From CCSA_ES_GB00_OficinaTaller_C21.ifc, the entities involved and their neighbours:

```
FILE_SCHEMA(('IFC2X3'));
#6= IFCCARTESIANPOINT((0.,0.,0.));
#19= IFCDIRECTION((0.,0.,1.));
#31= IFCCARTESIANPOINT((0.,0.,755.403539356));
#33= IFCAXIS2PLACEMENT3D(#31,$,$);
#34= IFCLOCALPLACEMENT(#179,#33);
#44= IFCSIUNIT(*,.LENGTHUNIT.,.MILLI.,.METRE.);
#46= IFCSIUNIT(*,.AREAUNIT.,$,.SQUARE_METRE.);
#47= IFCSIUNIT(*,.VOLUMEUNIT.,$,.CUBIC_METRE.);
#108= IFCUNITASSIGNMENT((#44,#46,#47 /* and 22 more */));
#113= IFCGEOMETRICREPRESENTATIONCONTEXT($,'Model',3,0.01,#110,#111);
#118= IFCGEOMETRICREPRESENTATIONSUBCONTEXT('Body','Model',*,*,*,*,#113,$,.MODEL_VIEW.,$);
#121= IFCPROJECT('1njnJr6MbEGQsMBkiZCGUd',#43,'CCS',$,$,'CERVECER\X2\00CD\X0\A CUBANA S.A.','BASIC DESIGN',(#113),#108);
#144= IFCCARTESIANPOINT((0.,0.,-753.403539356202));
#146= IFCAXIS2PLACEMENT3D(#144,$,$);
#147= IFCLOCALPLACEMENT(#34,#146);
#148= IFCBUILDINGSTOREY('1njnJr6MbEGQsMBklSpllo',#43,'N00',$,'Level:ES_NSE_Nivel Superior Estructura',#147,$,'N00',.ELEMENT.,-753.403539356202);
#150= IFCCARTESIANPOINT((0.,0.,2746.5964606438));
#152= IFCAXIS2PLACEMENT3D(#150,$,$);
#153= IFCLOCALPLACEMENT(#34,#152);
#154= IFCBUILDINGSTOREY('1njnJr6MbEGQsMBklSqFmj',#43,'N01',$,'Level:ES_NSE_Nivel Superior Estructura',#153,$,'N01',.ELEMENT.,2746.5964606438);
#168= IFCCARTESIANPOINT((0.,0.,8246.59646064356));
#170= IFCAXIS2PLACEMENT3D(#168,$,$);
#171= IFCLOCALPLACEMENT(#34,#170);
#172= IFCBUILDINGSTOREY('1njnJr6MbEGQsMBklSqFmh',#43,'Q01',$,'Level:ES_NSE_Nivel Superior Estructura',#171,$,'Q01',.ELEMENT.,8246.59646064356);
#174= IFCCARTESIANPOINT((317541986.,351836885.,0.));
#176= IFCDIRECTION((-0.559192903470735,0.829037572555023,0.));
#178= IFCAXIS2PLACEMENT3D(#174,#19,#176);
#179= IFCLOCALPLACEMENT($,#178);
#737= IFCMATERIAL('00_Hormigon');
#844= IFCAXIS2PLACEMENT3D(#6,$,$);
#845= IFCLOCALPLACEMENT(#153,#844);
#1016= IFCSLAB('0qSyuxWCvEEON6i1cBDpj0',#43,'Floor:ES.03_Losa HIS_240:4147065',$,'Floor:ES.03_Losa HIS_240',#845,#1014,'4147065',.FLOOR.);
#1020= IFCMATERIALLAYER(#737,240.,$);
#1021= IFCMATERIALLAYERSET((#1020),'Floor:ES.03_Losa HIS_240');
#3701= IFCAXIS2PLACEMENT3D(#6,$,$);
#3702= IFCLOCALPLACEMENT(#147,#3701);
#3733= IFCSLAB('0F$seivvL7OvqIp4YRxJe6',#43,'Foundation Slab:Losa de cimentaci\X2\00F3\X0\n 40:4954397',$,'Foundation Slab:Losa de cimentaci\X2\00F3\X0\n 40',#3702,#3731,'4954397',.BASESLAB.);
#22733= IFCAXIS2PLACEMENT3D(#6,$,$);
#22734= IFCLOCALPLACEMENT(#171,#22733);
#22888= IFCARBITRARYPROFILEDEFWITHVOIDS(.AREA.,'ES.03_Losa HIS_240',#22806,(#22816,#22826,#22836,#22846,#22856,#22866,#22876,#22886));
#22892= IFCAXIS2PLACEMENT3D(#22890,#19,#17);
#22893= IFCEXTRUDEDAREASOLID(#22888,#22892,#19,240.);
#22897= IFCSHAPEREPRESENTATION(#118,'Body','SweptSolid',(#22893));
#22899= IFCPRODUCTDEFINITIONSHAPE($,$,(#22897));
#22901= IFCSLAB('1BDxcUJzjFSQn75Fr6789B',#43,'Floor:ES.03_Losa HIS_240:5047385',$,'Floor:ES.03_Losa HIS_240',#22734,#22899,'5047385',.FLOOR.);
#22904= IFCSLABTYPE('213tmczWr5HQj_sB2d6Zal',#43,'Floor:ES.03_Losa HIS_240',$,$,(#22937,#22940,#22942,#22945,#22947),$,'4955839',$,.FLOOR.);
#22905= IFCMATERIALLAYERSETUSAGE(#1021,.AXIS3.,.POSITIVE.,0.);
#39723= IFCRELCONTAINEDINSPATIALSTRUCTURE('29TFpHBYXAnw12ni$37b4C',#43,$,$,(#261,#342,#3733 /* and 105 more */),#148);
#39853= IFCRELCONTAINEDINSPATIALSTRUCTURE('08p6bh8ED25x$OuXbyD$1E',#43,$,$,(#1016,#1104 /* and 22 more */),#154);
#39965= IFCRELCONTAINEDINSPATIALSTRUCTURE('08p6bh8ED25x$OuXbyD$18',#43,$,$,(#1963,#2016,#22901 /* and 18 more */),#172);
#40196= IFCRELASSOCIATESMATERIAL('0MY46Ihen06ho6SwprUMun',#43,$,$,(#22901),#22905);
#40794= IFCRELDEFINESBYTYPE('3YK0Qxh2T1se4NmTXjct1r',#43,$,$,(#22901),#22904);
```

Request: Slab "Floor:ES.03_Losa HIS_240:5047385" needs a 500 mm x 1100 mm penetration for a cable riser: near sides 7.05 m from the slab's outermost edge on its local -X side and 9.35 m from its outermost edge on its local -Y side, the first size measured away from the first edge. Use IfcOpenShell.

```python
import numpy as np
import ifcopenshell
import ifcopenshell.api.feature
import ifcopenshell.api.geometry
import ifcopenshell.api.root
import ifcopenshell.geom
import ifcopenshell.util.placement
import ifcopenshell.util.representation
import ifcopenshell.util.shape
import ifcopenshell.util.unit

model = ifcopenshell.open("CCSA_ES_GB00_OficinaTaller_C21.ifc")
unit_scale = ifcopenshell.util.unit.calculate_unit_scale(model)
settings = ifcopenshell.geom.settings()


def volume(element):
    """Net volume in cubic metres, openings subtracted."""
    shape = ifcopenshell.geom.create_shape(settings, element)
    return ifcopenshell.util.shape.get_volume(shape.geometry)


slab = model.by_guid("1BDxcUJzjFSQn75Fr6789B")
before = volume(slab)

# Extent in the slab's own axes, in metres. The edges named are its -X and -Y sides.
slab_shape = ifcopenshell.geom.create_shape(settings, slab)
vertices = ifcopenshell.util.shape.get_vertices(slab_shape.geometry)
x_min, y_min, bottom = vertices.min(axis=0)
top = vertices[:, 2].max()

opening = ifcopenshell.api.root.create_entity(model, ifc_class="IfcOpeningElement", name="Cable riser opening")
context = ifcopenshell.util.representation.get_context(model, "Model", "Body", "MODEL_VIEW")
width, depth = 0.5, 1.1
outline = [(0.0, 0.0), (width, 0.0), (width, depth), (0.0, depth), (0.0, 0.0)]
# Overshoot both faces by 50 mm so the cut is clean.
shape = ifcopenshell.api.geometry.add_slab_representation(
    model, context=context, depth=top - bottom + 0.1, polyline=outline
)
ifcopenshell.api.geometry.assign_representation(model, product=opening, representation=shape)

matrix = ifcopenshell.util.placement.get_local_placement(slab.ObjectPlacement)
matrix[:, 3] = matrix @ np.append(np.array([x_min + 7.05, y_min + 9.35, bottom - 0.05]) / unit_scale, 1.0)
ifcopenshell.api.geometry.edit_object_placement(model, product=opening, matrix=matrix, is_si=False)
ifcopenshell.api.feature.add_feature(model, feature=opening, element=slab)

after = volume(slab)

print(f"slab volume {before:.3f} -> {after:.3f} m3")

model.write("CCSA_ES_GB00_OficinaTaller_C21_edited.ifc")
```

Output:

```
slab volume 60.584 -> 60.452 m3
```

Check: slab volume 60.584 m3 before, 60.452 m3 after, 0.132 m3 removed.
